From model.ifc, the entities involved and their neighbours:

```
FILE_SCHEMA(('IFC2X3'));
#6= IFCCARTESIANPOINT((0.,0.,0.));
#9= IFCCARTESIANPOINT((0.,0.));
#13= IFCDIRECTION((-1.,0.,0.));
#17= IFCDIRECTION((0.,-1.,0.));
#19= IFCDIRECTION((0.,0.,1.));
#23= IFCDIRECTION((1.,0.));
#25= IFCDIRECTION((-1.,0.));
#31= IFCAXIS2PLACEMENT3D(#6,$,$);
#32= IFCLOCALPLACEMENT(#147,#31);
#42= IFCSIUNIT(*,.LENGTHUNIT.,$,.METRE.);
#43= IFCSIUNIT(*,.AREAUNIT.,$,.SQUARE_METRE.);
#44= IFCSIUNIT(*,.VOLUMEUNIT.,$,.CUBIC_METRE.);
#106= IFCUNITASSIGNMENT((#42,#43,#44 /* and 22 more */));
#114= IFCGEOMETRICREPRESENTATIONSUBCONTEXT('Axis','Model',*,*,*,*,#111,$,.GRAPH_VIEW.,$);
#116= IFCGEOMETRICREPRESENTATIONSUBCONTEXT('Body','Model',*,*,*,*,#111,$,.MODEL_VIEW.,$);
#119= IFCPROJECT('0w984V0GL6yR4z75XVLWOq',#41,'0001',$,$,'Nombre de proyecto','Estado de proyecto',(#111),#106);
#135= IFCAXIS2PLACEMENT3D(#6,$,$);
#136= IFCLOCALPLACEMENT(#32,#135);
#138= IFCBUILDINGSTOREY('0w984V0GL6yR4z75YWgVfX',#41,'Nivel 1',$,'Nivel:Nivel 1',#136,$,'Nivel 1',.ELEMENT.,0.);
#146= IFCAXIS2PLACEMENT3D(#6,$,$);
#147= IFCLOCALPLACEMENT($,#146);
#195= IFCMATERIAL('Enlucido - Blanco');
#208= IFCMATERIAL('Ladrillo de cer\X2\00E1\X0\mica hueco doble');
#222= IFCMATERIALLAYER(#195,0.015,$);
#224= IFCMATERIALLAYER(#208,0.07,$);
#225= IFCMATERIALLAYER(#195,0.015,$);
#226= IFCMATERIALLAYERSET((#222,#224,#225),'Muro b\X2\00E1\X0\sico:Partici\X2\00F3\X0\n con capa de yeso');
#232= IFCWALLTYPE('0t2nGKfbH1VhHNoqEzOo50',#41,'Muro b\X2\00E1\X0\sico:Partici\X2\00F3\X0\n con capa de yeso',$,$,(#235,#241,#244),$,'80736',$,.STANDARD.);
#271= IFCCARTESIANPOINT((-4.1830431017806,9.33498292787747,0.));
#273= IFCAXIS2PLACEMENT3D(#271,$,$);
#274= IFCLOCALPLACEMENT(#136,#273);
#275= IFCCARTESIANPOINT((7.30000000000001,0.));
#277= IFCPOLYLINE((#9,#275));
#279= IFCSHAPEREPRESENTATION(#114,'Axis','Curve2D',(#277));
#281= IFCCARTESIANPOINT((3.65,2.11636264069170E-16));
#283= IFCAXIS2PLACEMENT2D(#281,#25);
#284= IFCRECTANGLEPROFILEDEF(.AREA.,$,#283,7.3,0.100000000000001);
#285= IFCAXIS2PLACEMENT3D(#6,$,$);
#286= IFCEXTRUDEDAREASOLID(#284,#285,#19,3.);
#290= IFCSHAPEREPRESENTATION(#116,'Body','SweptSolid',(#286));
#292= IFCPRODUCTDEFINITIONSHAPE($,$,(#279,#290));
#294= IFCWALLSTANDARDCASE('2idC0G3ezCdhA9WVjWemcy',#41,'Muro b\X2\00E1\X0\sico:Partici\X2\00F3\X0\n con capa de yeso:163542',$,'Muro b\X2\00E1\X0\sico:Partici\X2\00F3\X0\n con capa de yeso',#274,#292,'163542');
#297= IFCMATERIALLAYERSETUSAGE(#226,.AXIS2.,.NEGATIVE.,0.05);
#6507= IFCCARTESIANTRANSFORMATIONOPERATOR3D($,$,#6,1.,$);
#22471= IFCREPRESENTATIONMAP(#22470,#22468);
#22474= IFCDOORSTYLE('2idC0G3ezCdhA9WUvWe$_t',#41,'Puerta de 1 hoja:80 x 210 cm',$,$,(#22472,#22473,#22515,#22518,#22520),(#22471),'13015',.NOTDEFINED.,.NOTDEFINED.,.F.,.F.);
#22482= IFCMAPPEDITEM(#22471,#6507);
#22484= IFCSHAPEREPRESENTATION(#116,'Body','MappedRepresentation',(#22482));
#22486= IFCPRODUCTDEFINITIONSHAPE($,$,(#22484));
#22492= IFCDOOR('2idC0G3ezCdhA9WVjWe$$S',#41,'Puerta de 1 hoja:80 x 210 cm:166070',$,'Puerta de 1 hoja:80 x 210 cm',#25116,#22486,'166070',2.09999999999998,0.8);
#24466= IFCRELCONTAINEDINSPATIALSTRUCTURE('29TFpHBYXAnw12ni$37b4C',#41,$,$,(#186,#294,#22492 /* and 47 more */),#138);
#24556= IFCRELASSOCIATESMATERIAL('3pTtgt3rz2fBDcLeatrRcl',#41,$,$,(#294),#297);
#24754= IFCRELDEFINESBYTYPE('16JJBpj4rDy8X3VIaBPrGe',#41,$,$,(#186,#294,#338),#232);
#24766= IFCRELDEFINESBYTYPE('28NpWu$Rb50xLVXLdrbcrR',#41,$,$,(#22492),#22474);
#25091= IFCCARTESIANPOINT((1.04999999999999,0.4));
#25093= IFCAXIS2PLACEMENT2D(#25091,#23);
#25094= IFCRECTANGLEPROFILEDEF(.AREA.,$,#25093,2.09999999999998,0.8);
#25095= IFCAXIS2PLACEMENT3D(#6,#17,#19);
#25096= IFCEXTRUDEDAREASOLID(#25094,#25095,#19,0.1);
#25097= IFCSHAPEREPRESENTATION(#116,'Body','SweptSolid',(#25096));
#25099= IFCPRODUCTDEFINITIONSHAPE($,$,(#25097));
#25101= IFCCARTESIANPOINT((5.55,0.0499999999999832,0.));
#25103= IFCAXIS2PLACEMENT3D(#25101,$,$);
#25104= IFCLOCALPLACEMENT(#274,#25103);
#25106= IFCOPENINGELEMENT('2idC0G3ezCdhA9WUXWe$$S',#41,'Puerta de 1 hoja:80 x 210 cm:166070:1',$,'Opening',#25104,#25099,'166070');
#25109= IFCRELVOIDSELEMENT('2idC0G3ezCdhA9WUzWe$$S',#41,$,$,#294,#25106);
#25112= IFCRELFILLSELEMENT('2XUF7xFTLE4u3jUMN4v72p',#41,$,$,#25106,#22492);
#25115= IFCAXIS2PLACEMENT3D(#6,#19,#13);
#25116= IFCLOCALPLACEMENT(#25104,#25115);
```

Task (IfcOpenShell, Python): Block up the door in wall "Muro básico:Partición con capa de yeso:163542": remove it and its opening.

```python
import ifcopenshell
import ifcopenshell.api.feature
import ifcopenshell.api.root
import ifcopenshell.geom
import ifcopenshell.util.shape

model = ifcopenshell.open("model.ifc")
settings = ifcopenshell.geom.settings()


def volume(element):
    """Net volume in cubic metres, openings subtracted."""
    shape = ifcopenshell.geom.create_shape(settings, element)
    return ifcopenshell.util.shape.get_volume(shape.geometry)


door = model.by_guid("2idC0G3ezCdhA9WVjWe$$S")
opening = door.FillsVoids[0].RelatingOpeningElement
wall = opening.VoidsElements[0].RelatingBuildingElement
before = volume(wall)

ifcopenshell.api.root.remove_product(model, product=door)
ifcopenshell.api.feature.remove_feature(model, feature=opening)

after = volume(wall)

print(f"wall volume {before:.3f} -> {after:.3f} m3")

model.write("model_updated.ifc")
```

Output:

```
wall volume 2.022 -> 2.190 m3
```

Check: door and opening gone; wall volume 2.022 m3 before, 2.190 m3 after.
